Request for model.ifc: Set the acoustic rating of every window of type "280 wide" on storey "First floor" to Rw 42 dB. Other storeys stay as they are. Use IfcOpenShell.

First a look at what the model holds.

```python
import ifcopenshell
import ifcopenshell.util.element

model = ifcopenshell.open("model.ifc")
print(model.schema)
storey = next(s for s in model.by_type("IfcBuildingStorey") if s.Name == "First floor")
windows = [e for e in ifcopenshell.util.element.get_decomposition(storey) if e.is_a("IfcWindow")]
seen = {}
for e in windows:
    element_type = ifcopenshell.util.element.get_type(e)
    key = (element_type.Name if element_type != e and element_type else None, ifcopenshell.util.element.get_pset(e, "Pset_WindowCommon", "AcousticRating"))
    seen[key] = seen.get(key, 0) + 1
for (name, value), count in sorted(seen.items(), key=str):
    print(count, "x", name, "|", value)
```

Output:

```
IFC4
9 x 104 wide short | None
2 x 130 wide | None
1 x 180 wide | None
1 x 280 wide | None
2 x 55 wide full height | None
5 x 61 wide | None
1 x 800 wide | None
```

```python
import ifcopenshell
import ifcopenshell.api.pset
import ifcopenshell.util.element

model = ifcopenshell.open("model.ifc")

storey = next(s for s in model.by_type("IfcBuildingStorey") if s.Name == "First floor")
windows = [e for e in ifcopenshell.util.element.get_decomposition(storey) if e.is_a("IfcWindow")]

count = 0
for e in windows:
    element_type = ifcopenshell.util.element.get_type(e)
    if element_type in (None, e) or element_type.Name != "280 wide":
        continue
    # add_pset returns the element's existing set when there is one.
    pset = ifcopenshell.api.pset.add_pset(model, product=e, name="Pset_WindowCommon")
    ifcopenshell.api.pset.edit_pset(model, pset=pset, properties={"AcousticRating": "Rw 42 dB"})
    count += 1

print(count, "windows updated")

model.write("model_rev.ifc")
```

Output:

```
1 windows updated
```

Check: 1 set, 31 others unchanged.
